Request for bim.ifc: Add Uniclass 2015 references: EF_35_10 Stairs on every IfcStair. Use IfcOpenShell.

First a look at what the model holds.

```python
import ifcopenshell

model = ifcopenshell.open("bim.ifc")
print(model.schema)
print("classifications:", [c.Name for c in model.by_type("IfcClassification")])
for ifc_class in ("IfcDoor", "IfcRoof", "IfcStair", "IfcWall", "IfcWindow"):
    print(ifc_class, len(model.by_type(ifc_class)))
```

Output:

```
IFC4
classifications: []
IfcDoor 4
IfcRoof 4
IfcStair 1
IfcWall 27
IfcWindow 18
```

```python
import ifcopenshell
import ifcopenshell.api.classification

model = ifcopenshell.open("bim.ifc")

system = ifcopenshell.api.classification.add_classification(model, classification="Uniclass 2015")

codes = {
    "IfcStair": ("EF_35_10", "Stairs"),
}
for ifc_class, (code, name) in codes.items():
    products = model.by_type(ifc_class)
    ifcopenshell.api.classification.add_reference(
        model, products=products, classification=system, identification=code, name=name
    )
    print(code, len(products))

model.write("bim_edited.ifc")
```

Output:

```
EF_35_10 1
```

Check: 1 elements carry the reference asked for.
